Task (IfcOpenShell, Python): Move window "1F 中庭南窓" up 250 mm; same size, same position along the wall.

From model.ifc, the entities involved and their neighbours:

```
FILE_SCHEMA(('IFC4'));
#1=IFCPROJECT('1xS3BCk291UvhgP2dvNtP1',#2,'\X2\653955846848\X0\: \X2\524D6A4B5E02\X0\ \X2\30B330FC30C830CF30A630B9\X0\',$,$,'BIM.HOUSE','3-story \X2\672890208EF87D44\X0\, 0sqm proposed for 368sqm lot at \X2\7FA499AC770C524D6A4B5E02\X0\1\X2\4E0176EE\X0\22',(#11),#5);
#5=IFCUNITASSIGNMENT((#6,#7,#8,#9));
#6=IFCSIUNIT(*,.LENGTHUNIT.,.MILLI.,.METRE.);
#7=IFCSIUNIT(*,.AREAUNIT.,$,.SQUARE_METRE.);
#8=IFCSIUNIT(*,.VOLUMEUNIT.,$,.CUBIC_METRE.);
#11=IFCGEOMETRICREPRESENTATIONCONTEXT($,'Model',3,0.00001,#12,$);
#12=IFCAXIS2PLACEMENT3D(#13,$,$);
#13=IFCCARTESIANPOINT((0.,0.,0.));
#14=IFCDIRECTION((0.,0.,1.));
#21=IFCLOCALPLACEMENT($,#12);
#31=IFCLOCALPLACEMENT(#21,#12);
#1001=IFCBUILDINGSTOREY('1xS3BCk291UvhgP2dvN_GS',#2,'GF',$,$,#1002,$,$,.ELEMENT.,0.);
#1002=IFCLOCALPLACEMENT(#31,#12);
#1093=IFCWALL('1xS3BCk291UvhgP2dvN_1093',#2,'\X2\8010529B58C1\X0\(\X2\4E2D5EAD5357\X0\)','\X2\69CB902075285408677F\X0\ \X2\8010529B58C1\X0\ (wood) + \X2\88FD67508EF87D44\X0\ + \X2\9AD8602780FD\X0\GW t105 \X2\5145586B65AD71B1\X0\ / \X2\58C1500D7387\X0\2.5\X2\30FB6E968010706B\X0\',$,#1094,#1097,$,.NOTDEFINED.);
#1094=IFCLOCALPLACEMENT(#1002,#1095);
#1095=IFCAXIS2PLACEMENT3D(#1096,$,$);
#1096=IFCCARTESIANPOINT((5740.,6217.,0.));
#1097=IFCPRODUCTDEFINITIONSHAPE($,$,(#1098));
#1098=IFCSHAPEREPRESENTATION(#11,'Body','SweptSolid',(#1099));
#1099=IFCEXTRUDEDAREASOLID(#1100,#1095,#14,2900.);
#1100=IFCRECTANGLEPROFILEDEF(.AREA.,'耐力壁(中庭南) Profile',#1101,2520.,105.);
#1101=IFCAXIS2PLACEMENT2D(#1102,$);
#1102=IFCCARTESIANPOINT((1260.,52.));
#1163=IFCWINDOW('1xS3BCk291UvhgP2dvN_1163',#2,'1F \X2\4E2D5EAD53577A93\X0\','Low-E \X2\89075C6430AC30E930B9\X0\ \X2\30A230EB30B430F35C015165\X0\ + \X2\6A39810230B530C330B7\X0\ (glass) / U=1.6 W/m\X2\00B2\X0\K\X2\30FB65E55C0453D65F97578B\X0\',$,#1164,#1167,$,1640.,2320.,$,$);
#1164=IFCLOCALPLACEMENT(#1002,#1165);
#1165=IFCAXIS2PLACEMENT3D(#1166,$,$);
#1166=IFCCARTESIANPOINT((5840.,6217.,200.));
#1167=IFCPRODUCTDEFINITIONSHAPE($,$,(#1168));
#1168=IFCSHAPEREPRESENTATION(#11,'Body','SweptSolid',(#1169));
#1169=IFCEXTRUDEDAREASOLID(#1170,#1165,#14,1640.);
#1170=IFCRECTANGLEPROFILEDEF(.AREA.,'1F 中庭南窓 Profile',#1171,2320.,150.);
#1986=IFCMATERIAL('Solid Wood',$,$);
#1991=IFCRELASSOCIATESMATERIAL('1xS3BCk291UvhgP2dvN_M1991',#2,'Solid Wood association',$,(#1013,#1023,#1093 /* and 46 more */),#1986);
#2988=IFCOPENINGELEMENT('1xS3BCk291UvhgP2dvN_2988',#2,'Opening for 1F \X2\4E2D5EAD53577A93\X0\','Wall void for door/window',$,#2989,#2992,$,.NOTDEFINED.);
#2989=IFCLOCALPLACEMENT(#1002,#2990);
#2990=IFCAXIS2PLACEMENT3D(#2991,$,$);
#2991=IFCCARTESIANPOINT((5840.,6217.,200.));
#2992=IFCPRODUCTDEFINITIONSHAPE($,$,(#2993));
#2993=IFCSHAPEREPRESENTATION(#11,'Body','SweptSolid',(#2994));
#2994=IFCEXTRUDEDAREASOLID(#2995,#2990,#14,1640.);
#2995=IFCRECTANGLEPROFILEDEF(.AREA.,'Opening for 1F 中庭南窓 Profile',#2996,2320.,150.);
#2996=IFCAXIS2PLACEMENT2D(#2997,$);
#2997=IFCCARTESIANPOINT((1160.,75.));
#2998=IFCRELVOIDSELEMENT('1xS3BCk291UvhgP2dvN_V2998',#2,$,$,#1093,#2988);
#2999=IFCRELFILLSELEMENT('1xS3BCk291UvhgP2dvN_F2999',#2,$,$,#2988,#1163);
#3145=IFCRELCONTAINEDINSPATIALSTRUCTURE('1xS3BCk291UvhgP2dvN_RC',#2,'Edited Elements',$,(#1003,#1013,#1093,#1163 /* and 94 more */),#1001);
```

```python
import numpy as np
import ifcopenshell
import ifcopenshell.api.geometry
import ifcopenshell.util.placement
import ifcopenshell.util.unit

model = ifcopenshell.open("model.ifc")
unit_scale = ifcopenshell.util.unit.calculate_unit_scale(model)

window = model.by_guid("1xS3BCk291UvhgP2dvN_1163")
opening = window.FillsVoids[0].RelatingOpeningElement
dz = 250.0

shift = np.array([0.0, 0.0, dz])
# The window is not placed relative to its opening, so move both.
for product in (opening, window):
    matrix = ifcopenshell.util.placement.get_local_placement(product.ObjectPlacement)
    matrix[:3, 3] += shift
    ifcopenshell.api.geometry.edit_object_placement(model, product=product, matrix=matrix, is_si=False)

print(f"moved by {dz * unit_scale:+.3f} m")

model.write("model_rev.ifc")
```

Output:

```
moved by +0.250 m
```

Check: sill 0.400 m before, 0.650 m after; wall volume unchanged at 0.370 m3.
